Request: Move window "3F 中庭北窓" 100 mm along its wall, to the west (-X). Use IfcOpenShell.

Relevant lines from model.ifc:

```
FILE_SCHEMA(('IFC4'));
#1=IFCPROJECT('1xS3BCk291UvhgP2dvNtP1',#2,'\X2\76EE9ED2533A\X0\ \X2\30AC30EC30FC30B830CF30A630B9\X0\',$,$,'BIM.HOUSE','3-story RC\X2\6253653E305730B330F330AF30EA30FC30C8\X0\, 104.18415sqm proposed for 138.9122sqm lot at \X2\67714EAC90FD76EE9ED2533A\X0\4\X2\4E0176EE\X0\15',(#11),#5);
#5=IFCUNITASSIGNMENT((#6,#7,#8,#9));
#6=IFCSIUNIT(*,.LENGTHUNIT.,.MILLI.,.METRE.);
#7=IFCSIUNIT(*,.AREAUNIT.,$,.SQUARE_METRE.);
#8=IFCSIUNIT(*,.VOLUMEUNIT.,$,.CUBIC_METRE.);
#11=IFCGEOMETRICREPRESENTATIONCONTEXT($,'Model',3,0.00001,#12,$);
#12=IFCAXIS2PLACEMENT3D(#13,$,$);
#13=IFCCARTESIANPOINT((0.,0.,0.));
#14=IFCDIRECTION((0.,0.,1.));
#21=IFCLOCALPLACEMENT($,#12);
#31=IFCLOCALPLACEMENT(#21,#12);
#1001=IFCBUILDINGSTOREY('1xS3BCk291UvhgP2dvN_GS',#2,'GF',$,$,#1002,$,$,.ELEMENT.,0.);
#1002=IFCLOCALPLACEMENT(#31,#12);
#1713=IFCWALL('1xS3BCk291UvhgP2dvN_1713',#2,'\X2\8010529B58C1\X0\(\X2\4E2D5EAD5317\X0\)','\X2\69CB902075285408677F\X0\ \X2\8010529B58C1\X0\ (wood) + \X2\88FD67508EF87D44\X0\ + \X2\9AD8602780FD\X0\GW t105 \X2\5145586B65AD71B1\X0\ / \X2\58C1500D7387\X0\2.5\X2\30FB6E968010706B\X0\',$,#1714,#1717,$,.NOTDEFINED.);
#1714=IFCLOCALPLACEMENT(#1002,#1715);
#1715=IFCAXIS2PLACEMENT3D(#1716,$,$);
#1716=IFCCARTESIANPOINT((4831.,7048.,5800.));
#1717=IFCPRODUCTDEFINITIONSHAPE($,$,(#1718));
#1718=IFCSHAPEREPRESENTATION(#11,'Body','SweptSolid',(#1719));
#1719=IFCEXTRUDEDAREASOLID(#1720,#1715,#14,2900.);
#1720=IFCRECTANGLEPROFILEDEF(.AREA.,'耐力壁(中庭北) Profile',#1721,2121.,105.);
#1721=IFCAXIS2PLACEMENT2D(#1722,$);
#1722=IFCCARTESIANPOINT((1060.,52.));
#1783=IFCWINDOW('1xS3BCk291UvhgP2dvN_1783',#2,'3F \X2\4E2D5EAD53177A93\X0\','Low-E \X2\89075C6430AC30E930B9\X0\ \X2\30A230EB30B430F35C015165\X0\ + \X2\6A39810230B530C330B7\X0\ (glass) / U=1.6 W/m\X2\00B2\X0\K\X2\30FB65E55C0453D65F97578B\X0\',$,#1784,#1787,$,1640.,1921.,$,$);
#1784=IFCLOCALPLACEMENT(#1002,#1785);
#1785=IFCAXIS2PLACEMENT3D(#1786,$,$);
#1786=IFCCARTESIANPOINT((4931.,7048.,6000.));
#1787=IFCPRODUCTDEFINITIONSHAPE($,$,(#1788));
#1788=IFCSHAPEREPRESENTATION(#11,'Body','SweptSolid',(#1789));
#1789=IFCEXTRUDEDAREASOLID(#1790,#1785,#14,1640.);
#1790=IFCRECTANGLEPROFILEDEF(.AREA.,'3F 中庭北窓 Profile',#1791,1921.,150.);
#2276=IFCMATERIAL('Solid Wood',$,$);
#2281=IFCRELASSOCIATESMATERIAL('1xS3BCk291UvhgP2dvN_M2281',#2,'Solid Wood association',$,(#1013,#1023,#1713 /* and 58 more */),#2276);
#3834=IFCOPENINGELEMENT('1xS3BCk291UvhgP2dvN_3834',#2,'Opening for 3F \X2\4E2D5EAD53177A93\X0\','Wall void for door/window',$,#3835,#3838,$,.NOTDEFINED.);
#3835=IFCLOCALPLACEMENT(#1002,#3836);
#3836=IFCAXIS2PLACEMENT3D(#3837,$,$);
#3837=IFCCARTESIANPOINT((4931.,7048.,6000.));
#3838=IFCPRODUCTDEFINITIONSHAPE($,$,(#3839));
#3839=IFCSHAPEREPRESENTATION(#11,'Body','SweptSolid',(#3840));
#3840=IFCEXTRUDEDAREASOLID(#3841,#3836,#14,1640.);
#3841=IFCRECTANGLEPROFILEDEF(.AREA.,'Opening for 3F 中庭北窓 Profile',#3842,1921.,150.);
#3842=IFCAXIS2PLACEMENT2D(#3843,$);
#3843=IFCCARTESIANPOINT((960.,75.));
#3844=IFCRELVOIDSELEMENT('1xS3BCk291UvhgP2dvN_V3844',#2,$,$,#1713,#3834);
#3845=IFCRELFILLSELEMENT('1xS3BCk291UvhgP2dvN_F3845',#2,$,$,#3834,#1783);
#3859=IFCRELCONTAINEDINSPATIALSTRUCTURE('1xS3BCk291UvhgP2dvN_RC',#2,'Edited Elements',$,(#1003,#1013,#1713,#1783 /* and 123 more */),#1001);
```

```python
import ifcopenshell
import ifcopenshell.api.geometry
import ifcopenshell.util.placement

model = ifcopenshell.open("model.ifc")

window = model.by_guid("1xS3BCk291UvhgP2dvN_1783")
opening = window.FillsVoids[0].RelatingOpeningElement
wall = opening.VoidsElements[0].RelatingBuildingElement

wall_matrix = ifcopenshell.util.placement.get_local_placement(wall.ObjectPlacement)
shift = wall_matrix[:3, 0] * -100.0
before = ifcopenshell.util.placement.get_local_placement(window.ObjectPlacement)[:3, 3].copy()

# The window is not placed relative to its opening, so move both.
for product in (opening, window):
    matrix = ifcopenshell.util.placement.get_local_placement(product.ObjectPlacement)
    matrix[:3, 3] += shift
    ifcopenshell.api.geometry.edit_object_placement(model, product=product, matrix=matrix, is_si=False)

after = ifcopenshell.util.placement.get_local_placement(window.ObjectPlacement)[:3, 3]
print("window moved by", (after - before).round(3) + 0.0)

model.write("model_updated.ifc")
```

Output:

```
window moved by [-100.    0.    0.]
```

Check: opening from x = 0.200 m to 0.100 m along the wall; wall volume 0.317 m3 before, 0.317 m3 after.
